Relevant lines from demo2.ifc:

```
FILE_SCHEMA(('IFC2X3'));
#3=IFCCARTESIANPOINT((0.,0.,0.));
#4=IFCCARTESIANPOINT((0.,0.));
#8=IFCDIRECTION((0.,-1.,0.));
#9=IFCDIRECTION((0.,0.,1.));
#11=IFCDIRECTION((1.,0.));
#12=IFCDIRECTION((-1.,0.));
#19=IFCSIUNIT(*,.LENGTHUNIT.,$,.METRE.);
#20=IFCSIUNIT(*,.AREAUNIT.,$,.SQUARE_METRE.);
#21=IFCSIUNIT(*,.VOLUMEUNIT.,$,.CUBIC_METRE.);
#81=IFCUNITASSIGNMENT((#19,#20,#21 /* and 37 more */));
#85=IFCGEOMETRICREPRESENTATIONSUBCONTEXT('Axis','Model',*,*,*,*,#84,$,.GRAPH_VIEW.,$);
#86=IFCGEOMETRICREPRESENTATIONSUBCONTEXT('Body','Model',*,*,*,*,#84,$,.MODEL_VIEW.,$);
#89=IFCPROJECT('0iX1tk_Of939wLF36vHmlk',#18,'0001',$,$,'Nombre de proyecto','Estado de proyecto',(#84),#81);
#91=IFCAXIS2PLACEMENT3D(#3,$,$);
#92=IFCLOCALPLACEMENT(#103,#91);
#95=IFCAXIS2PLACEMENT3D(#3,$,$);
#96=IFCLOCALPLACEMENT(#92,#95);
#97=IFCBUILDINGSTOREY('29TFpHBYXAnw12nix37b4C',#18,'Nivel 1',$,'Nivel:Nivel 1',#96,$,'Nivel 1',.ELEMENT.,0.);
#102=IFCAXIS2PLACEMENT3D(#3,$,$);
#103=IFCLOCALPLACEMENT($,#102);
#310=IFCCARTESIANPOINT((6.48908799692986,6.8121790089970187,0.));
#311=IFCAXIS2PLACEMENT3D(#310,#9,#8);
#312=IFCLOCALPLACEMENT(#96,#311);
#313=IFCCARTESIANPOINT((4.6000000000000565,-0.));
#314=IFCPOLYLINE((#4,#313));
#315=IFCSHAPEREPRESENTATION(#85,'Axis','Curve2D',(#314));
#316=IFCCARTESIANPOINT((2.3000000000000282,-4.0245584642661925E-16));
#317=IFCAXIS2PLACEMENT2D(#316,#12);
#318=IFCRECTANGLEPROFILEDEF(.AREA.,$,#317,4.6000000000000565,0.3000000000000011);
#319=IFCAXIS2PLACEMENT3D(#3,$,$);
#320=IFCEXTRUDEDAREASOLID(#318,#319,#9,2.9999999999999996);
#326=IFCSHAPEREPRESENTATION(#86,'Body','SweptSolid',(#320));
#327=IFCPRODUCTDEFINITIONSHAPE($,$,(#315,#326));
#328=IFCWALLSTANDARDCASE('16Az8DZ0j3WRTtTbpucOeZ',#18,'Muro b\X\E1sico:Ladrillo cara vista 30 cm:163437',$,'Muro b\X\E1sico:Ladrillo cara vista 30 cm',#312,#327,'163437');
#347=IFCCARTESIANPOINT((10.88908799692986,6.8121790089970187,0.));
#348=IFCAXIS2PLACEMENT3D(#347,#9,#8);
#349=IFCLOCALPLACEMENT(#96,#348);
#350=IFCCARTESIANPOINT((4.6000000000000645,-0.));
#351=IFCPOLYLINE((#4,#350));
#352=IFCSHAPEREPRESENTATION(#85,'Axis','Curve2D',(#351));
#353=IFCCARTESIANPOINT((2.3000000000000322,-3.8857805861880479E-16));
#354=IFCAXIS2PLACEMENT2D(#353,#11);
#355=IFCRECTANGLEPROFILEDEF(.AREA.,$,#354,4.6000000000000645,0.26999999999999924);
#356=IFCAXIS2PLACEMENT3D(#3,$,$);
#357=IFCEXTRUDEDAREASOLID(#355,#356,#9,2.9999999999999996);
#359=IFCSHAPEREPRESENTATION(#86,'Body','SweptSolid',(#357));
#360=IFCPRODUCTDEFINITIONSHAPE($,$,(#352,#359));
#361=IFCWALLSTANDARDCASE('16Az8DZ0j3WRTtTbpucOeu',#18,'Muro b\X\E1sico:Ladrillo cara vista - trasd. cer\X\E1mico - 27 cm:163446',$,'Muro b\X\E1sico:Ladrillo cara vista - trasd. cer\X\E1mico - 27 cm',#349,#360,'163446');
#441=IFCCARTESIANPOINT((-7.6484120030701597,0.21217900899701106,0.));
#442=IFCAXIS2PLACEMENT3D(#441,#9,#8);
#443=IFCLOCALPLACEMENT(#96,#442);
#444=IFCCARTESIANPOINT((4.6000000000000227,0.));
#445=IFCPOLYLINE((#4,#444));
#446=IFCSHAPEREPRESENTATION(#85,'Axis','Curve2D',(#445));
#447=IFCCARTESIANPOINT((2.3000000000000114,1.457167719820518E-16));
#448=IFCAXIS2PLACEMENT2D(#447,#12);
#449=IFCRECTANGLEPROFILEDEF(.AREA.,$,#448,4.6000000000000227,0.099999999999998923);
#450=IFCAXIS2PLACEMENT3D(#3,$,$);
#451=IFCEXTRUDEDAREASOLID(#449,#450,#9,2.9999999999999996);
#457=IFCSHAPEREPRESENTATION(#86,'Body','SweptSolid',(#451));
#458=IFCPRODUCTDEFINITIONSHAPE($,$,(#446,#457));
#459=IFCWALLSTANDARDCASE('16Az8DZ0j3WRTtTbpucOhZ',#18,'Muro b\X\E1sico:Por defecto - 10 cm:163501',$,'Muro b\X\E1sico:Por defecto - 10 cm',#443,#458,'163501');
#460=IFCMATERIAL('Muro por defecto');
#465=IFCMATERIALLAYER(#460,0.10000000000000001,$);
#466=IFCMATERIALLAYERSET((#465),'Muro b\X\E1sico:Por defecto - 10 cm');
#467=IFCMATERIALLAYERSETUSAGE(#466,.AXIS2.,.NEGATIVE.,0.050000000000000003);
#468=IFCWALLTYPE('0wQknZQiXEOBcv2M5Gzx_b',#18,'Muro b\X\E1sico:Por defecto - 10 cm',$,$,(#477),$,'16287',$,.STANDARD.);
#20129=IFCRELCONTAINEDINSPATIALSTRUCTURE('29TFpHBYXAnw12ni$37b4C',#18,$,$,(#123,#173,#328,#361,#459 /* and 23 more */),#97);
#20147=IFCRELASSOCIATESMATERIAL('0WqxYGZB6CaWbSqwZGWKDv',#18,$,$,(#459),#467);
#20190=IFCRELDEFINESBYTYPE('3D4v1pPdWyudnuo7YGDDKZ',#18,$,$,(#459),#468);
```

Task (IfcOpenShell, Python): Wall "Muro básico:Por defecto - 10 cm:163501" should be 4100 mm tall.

```python
import ifcopenshell
import ifcopenshell.geom
import ifcopenshell.util.representation
import ifcopenshell.util.shape

model = ifcopenshell.open("demo2.ifc")
settings = ifcopenshell.geom.settings()


def volume(element):
    """Net volume in cubic metres, openings subtracted."""
    shape = ifcopenshell.geom.create_shape(settings, element)
    return ifcopenshell.util.shape.get_volume(shape.geometry)


wall = model.by_guid("16Az8DZ0j3WRTtTbpucOhZ")
before = volume(wall)

body = ifcopenshell.util.representation.get_representation(wall, "Model", "Body")
solid = body.Items[0]
old_height = solid.Depth
solid.Depth = 4.1
after = volume(wall)

print(f"height {old_height:g} -> {solid.Depth:g}, volume {before:.3f} -> {after:.3f} m3")

model.write("demo2_edited.ifc")
```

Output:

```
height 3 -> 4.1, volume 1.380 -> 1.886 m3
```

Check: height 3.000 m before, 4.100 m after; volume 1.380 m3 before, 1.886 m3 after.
